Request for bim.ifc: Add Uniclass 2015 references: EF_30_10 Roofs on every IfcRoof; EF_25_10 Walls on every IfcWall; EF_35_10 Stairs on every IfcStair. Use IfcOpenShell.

First a look at what the model holds.

```python
import ifcopenshell

model = ifcopenshell.open("bim.ifc")
print(model.schema)
print("classifications:", [c.Name for c in model.by_type("IfcClassification")])
for ifc_class in ("IfcDoor", "IfcRoof", "IfcStair", "IfcWall", "IfcWindow"):
    print(ifc_class, len(model.by_type(ifc_class)))
```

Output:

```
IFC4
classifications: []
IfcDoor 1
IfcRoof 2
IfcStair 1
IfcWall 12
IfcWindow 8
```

```python
import ifcopenshell
import ifcopenshell.api.classification

model = ifcopenshell.open("bim.ifc")

system = ifcopenshell.api.classification.add_classification(model, classification="Uniclass 2015")

codes = {
    "IfcRoof": ("EF_30_10", "Roofs"),
    "IfcWall": ("EF_25_10", "Walls"),
    "IfcStair": ("EF_35_10", "Stairs"),
}
for ifc_class, (code, name) in codes.items():
    products = model.by_type(ifc_class)
    ifcopenshell.api.classification.add_reference(
        model, products=products, classification=system, identification=code, name=name
    )
    print(code, len(products))

model.write("bim_updated.ifc")
```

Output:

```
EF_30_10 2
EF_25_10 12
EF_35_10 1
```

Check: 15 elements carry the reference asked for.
